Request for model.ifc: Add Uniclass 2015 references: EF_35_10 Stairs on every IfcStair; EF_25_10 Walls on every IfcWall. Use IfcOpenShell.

First a look at what the model holds.

```python
import ifcopenshell

model = ifcopenshell.open("model.ifc")
print(model.schema)
print("classifications:", [c.Name for c in model.by_type("IfcClassification")])
for ifc_class in ("IfcDoor", "IfcRoof", "IfcStair", "IfcWall", "IfcWindow"):
    print(ifc_class, len(model.by_type(ifc_class)))
```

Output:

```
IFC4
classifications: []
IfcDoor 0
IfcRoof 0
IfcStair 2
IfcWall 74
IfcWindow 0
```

```python
import ifcopenshell
import ifcopenshell.api.classification

model = ifcopenshell.open("model.ifc")

system = ifcopenshell.api.classification.add_classification(model, classification="Uniclass 2015")

codes = {
    "IfcStair": ("EF_35_10", "Stairs"),
    "IfcWall": ("EF_25_10", "Walls"),
}
for ifc_class, (code, name) in codes.items():
    products = model.by_type(ifc_class)
    ifcopenshell.api.classification.add_reference(
        model, products=products, classification=system, identification=code, name=name
    )
    print(code, len(products))

model.write("model_rev.ifc")
```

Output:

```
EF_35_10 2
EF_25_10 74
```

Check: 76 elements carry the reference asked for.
